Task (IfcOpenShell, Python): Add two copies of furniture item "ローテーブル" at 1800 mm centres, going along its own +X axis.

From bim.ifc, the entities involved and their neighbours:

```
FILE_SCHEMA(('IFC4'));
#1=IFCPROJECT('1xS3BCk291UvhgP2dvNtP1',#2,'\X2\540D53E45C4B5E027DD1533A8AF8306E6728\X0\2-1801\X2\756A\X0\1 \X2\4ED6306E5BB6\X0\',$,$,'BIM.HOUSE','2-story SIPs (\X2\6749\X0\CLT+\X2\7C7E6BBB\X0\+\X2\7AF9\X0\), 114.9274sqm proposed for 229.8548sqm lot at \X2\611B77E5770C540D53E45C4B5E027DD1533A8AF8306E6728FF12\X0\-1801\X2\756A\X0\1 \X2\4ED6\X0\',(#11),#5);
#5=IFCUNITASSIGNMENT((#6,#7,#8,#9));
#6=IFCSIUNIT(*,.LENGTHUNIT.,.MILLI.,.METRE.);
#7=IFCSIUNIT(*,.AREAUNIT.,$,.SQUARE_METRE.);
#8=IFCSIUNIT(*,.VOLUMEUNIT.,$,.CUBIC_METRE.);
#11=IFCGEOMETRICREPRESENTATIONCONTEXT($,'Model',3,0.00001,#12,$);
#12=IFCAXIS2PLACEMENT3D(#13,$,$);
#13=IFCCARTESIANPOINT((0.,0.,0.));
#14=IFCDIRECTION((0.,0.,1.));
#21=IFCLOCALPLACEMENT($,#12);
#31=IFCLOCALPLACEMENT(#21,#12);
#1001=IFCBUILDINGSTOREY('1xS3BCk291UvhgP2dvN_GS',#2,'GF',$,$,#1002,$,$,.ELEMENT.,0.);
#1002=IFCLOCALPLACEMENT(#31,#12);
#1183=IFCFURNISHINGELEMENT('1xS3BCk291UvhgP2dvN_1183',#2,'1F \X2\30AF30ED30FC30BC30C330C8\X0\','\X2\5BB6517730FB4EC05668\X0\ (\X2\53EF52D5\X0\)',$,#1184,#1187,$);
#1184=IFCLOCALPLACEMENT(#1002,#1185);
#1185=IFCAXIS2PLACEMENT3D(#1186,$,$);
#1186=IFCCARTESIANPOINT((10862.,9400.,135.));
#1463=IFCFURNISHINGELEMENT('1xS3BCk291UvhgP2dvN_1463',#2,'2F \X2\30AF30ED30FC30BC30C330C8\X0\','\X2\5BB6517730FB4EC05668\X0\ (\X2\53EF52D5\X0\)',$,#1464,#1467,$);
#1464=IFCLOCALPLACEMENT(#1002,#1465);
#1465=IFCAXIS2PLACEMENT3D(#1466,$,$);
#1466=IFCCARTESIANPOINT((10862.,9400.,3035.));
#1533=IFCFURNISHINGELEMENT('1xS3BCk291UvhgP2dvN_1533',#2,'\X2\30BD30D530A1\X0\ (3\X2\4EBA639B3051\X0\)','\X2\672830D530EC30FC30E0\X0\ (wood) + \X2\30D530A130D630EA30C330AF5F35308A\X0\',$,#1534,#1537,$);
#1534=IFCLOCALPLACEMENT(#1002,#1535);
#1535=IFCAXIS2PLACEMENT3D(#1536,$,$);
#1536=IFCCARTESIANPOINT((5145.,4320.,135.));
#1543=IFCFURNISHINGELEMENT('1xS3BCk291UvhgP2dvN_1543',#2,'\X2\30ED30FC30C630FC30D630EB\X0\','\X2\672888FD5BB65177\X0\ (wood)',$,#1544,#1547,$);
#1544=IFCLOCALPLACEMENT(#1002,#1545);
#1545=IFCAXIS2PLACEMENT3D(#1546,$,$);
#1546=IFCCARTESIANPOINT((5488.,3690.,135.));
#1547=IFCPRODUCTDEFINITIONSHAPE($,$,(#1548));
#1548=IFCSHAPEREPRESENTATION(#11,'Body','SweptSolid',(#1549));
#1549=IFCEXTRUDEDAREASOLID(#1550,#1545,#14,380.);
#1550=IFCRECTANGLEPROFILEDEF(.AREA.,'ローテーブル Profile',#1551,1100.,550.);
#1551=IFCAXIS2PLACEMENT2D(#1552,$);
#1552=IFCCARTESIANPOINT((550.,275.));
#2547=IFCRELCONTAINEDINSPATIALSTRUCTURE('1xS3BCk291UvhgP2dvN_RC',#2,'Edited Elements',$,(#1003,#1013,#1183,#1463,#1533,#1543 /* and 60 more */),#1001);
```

```python
import ifcopenshell
import ifcopenshell.api.geometry
import ifcopenshell.api.root
import ifcopenshell.util.element
import ifcopenshell.util.placement
import ifcopenshell.util.unit

model = ifcopenshell.open("bim.ifc")
unit_scale = ifcopenshell.util.unit.calculate_unit_scale(model)


def reuse_history(source, copy):
    """copy_class also copies each property set's owner history, people and application; keep the originals."""
    for rel in copy.IsDefinedBy:
        if rel.is_a("IfcRelDefinesByProperties") and (history := rel.RelatingPropertyDefinition.OwnerHistory):
            rel.RelatingPropertyDefinition.OwnerHistory = source.OwnerHistory
            ifcopenshell.util.element.remove_deep2(model, history)


source = model.by_guid("1xS3BCk291UvhgP2dvN_1543")
base = ifcopenshell.util.placement.get_local_placement(source.ObjectPlacement)
step = base[:3, 0] * 1.8 / unit_scale

for i in range(1, 3):
    copy = ifcopenshell.api.root.copy_class(model, product=source)
    copy.Representation = ifcopenshell.util.element.copy_deep(
        model, source.Representation, exclude=["IfcGeometricRepresentationContext", "IfcRepresentationMap"]
    )
    reuse_history(source, copy)
    matrix = base.copy()
    matrix[:3, 3] += i * step
    print("added at", matrix[:3, 3].round(3) + 0.0)
    ifcopenshell.api.geometry.edit_object_placement(model, product=copy, matrix=matrix, is_si=False)

model.write("bim_rev.ifc")
```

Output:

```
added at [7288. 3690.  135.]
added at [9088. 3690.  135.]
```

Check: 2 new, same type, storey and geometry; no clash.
